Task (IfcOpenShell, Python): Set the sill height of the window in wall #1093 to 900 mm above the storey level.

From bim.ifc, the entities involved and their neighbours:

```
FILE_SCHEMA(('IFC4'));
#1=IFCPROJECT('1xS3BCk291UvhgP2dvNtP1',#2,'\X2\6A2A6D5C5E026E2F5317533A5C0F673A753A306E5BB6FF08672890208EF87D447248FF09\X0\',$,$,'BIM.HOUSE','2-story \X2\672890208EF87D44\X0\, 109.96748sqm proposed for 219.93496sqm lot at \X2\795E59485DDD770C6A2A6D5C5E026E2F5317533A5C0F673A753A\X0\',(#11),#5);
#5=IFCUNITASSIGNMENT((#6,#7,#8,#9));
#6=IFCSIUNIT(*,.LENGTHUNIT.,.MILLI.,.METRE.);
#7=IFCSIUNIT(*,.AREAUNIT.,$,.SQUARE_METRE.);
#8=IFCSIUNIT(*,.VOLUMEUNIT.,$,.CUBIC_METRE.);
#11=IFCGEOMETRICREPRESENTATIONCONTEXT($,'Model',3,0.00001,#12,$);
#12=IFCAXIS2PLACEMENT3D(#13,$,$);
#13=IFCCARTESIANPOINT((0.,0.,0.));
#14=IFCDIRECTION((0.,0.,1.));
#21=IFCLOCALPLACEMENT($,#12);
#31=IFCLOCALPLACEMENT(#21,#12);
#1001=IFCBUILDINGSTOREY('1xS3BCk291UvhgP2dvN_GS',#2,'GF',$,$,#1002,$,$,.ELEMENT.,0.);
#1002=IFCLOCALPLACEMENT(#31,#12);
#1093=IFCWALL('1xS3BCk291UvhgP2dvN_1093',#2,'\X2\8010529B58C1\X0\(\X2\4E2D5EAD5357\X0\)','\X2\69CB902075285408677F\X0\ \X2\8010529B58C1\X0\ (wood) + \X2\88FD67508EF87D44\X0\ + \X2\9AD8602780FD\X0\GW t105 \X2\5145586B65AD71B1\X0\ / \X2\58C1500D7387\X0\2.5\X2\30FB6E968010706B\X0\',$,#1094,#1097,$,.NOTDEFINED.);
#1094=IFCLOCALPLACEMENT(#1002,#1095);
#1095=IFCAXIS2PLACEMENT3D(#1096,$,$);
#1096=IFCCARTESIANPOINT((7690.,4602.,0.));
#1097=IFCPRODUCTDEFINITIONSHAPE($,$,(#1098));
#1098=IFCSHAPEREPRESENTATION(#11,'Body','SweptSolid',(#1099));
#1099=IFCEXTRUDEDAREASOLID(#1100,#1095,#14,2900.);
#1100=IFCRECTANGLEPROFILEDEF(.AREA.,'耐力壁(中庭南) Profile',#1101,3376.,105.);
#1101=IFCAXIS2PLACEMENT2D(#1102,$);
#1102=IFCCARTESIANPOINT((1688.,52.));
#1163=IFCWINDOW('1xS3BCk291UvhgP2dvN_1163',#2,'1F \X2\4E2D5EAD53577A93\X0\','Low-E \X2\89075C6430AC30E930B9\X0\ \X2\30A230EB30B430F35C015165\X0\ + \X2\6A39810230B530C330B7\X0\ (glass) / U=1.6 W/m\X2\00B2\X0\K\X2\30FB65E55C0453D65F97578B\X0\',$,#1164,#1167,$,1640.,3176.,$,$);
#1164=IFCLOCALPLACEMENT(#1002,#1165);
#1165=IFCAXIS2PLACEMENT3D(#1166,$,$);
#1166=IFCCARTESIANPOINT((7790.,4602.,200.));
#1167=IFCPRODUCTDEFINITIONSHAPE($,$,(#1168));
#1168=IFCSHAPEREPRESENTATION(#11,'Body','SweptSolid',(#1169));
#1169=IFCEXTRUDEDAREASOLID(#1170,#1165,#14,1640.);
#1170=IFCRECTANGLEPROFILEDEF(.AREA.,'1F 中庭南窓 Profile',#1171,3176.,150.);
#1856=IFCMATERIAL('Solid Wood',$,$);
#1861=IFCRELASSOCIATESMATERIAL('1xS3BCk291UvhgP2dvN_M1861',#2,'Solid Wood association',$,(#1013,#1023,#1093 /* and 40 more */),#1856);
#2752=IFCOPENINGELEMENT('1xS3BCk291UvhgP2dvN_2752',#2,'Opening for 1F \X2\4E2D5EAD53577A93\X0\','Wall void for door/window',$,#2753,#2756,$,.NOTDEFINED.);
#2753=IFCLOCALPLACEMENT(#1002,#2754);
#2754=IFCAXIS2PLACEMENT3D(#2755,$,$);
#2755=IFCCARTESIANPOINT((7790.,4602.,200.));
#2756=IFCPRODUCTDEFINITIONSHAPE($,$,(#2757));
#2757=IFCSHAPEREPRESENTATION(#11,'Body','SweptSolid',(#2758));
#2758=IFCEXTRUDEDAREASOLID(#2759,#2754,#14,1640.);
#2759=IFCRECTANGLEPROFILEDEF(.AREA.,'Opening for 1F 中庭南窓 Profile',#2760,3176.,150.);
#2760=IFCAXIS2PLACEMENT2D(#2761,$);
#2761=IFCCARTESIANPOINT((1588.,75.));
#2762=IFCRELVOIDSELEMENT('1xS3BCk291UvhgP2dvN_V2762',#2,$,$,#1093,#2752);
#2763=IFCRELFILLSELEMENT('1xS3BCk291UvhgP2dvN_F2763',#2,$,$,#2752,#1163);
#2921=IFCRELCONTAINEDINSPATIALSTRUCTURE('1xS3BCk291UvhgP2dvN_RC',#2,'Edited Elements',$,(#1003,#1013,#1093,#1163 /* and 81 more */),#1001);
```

```python
import numpy as np
import ifcopenshell
import ifcopenshell.api.geometry
import ifcopenshell.geom
import ifcopenshell.util.element
import ifcopenshell.util.placement
import ifcopenshell.util.shape
import ifcopenshell.util.unit

model = ifcopenshell.open("bim.ifc")
unit_scale = ifcopenshell.util.unit.calculate_unit_scale(model)

window = model.by_id(1163)
opening = window.FillsVoids[0].RelatingOpeningElement
storey = ifcopenshell.util.element.get_container(window, ifc_class="IfcBuildingStorey")
level = ifcopenshell.util.placement.get_local_placement(storey.ObjectPlacement)[2, 3]

# The opening's origin need not be at the sill, so measure its lowest point.
shape = ifcopenshell.geom.create_shape(ifcopenshell.geom.settings(), opening)
bottom = ifcopenshell.util.shape.get_shape_bottom_elevation(shape, shape.geometry) / unit_scale
dz = level + 900.0 - bottom

shift = np.array([0.0, 0.0, dz])
# The window is not placed relative to its opening, so move both.
for product in (opening, window):
    matrix = ifcopenshell.util.placement.get_local_placement(product.ObjectPlacement)
    matrix[:3, 3] += shift
    ifcopenshell.api.geometry.edit_object_placement(model, product=product, matrix=matrix, is_si=False)

print(f"moved by {dz * unit_scale:+.3f} m")

model.write("bim-out.ifc")
```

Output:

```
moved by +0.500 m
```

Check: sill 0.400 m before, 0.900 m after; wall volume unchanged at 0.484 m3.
